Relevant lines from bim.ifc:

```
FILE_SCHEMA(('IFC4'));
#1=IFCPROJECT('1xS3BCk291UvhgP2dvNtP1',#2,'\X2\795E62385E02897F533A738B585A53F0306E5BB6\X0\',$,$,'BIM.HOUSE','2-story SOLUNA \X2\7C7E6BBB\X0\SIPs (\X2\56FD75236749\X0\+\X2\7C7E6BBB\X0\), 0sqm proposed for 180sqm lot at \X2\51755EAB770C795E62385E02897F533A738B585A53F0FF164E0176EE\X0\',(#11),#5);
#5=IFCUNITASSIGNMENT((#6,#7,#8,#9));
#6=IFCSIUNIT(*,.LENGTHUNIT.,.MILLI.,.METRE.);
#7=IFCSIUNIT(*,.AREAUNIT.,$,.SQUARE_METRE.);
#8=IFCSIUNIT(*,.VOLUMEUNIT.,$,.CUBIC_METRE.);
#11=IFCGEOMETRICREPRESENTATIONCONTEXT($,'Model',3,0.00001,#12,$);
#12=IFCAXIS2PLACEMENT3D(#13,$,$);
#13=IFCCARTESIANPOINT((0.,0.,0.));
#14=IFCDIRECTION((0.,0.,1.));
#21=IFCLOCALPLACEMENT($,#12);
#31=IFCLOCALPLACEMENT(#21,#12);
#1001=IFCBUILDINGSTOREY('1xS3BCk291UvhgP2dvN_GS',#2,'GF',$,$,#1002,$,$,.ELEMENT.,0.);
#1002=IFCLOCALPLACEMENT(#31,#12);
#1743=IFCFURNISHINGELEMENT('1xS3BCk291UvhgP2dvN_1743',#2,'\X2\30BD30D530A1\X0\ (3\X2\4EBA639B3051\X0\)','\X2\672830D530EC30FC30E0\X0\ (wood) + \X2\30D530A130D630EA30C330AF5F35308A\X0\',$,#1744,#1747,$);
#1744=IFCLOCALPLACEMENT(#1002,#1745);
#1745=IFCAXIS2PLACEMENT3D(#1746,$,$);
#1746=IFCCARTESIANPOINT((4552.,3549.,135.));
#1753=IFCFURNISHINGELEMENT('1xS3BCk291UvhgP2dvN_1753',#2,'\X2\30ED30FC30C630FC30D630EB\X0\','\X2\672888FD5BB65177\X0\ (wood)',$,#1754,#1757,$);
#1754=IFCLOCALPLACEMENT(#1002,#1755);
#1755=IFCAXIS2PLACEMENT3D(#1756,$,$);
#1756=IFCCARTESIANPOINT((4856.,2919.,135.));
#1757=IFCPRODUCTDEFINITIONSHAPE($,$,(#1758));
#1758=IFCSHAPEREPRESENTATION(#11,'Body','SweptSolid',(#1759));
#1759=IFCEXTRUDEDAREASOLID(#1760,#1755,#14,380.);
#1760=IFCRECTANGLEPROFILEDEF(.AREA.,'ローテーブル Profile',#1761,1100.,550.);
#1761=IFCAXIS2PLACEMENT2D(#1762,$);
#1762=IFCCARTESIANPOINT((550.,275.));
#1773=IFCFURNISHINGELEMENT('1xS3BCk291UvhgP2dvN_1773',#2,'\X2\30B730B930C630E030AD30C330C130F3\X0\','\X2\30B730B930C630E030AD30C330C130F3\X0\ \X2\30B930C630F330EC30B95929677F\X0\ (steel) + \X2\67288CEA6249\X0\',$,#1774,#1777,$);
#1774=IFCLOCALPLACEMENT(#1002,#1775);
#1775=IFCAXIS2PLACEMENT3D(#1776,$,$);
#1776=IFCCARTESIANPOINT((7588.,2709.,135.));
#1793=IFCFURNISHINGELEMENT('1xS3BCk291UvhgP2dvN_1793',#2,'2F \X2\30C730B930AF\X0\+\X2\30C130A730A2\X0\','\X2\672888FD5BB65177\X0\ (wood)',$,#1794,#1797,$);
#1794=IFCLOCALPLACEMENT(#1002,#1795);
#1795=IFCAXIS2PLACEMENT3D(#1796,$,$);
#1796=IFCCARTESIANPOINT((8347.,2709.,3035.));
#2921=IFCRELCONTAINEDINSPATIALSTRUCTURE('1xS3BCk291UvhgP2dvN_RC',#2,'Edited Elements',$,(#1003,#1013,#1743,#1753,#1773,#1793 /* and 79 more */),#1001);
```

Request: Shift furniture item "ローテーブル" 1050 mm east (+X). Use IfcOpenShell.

```python
import ifcopenshell
import ifcopenshell.api.geometry
import ifcopenshell.util.placement
import ifcopenshell.util.unit

model = ifcopenshell.open("bim.ifc")
unit_scale = ifcopenshell.util.unit.calculate_unit_scale(model)

item = model.by_guid("1xS3BCk291UvhgP2dvN_1753")
matrix = ifcopenshell.util.placement.get_local_placement(item.ObjectPlacement)
matrix[0, 3] += 1.05 / unit_scale
ifcopenshell.api.geometry.edit_object_placement(model, product=item, matrix=matrix, is_si=False)

print(ifcopenshell.util.placement.get_local_placement(item.ObjectPlacement).round(3) + 0.0)

model.write("bim_v2.ifc")
```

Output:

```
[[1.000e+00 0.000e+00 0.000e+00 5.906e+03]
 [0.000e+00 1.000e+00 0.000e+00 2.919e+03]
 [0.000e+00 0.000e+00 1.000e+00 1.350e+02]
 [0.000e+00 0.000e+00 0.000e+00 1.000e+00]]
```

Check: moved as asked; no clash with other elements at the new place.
